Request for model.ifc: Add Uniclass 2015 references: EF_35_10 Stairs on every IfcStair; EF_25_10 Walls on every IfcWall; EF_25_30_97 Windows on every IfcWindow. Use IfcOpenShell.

First a look at what the model holds.

```python
import ifcopenshell

model = ifcopenshell.open("model.ifc")
print(model.schema)
print("classifications:", [c.Name for c in model.by_type("IfcClassification")])
for ifc_class in ("IfcDoor", "IfcRoof", "IfcStair", "IfcWall", "IfcWindow"):
    print(ifc_class, len(model.by_type(ifc_class)))
```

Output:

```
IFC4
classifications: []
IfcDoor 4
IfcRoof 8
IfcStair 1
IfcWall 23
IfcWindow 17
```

```python
import ifcopenshell
import ifcopenshell.api.classification

model = ifcopenshell.open("model.ifc")

system = ifcopenshell.api.classification.add_classification(model, classification="Uniclass 2015")

codes = {
    "IfcStair": ("EF_35_10", "Stairs"),
    "IfcWall": ("EF_25_10", "Walls"),
    "IfcWindow": ("EF_25_30_97", "Windows"),
}
for ifc_class, (code, name) in codes.items():
    products = model.by_type(ifc_class)
    ifcopenshell.api.classification.add_reference(
        model, products=products, classification=system, identification=code, name=name
    )
    print(code, len(products))

model.write("model-out.ifc")
```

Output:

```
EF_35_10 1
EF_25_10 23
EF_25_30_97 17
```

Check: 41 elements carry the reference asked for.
